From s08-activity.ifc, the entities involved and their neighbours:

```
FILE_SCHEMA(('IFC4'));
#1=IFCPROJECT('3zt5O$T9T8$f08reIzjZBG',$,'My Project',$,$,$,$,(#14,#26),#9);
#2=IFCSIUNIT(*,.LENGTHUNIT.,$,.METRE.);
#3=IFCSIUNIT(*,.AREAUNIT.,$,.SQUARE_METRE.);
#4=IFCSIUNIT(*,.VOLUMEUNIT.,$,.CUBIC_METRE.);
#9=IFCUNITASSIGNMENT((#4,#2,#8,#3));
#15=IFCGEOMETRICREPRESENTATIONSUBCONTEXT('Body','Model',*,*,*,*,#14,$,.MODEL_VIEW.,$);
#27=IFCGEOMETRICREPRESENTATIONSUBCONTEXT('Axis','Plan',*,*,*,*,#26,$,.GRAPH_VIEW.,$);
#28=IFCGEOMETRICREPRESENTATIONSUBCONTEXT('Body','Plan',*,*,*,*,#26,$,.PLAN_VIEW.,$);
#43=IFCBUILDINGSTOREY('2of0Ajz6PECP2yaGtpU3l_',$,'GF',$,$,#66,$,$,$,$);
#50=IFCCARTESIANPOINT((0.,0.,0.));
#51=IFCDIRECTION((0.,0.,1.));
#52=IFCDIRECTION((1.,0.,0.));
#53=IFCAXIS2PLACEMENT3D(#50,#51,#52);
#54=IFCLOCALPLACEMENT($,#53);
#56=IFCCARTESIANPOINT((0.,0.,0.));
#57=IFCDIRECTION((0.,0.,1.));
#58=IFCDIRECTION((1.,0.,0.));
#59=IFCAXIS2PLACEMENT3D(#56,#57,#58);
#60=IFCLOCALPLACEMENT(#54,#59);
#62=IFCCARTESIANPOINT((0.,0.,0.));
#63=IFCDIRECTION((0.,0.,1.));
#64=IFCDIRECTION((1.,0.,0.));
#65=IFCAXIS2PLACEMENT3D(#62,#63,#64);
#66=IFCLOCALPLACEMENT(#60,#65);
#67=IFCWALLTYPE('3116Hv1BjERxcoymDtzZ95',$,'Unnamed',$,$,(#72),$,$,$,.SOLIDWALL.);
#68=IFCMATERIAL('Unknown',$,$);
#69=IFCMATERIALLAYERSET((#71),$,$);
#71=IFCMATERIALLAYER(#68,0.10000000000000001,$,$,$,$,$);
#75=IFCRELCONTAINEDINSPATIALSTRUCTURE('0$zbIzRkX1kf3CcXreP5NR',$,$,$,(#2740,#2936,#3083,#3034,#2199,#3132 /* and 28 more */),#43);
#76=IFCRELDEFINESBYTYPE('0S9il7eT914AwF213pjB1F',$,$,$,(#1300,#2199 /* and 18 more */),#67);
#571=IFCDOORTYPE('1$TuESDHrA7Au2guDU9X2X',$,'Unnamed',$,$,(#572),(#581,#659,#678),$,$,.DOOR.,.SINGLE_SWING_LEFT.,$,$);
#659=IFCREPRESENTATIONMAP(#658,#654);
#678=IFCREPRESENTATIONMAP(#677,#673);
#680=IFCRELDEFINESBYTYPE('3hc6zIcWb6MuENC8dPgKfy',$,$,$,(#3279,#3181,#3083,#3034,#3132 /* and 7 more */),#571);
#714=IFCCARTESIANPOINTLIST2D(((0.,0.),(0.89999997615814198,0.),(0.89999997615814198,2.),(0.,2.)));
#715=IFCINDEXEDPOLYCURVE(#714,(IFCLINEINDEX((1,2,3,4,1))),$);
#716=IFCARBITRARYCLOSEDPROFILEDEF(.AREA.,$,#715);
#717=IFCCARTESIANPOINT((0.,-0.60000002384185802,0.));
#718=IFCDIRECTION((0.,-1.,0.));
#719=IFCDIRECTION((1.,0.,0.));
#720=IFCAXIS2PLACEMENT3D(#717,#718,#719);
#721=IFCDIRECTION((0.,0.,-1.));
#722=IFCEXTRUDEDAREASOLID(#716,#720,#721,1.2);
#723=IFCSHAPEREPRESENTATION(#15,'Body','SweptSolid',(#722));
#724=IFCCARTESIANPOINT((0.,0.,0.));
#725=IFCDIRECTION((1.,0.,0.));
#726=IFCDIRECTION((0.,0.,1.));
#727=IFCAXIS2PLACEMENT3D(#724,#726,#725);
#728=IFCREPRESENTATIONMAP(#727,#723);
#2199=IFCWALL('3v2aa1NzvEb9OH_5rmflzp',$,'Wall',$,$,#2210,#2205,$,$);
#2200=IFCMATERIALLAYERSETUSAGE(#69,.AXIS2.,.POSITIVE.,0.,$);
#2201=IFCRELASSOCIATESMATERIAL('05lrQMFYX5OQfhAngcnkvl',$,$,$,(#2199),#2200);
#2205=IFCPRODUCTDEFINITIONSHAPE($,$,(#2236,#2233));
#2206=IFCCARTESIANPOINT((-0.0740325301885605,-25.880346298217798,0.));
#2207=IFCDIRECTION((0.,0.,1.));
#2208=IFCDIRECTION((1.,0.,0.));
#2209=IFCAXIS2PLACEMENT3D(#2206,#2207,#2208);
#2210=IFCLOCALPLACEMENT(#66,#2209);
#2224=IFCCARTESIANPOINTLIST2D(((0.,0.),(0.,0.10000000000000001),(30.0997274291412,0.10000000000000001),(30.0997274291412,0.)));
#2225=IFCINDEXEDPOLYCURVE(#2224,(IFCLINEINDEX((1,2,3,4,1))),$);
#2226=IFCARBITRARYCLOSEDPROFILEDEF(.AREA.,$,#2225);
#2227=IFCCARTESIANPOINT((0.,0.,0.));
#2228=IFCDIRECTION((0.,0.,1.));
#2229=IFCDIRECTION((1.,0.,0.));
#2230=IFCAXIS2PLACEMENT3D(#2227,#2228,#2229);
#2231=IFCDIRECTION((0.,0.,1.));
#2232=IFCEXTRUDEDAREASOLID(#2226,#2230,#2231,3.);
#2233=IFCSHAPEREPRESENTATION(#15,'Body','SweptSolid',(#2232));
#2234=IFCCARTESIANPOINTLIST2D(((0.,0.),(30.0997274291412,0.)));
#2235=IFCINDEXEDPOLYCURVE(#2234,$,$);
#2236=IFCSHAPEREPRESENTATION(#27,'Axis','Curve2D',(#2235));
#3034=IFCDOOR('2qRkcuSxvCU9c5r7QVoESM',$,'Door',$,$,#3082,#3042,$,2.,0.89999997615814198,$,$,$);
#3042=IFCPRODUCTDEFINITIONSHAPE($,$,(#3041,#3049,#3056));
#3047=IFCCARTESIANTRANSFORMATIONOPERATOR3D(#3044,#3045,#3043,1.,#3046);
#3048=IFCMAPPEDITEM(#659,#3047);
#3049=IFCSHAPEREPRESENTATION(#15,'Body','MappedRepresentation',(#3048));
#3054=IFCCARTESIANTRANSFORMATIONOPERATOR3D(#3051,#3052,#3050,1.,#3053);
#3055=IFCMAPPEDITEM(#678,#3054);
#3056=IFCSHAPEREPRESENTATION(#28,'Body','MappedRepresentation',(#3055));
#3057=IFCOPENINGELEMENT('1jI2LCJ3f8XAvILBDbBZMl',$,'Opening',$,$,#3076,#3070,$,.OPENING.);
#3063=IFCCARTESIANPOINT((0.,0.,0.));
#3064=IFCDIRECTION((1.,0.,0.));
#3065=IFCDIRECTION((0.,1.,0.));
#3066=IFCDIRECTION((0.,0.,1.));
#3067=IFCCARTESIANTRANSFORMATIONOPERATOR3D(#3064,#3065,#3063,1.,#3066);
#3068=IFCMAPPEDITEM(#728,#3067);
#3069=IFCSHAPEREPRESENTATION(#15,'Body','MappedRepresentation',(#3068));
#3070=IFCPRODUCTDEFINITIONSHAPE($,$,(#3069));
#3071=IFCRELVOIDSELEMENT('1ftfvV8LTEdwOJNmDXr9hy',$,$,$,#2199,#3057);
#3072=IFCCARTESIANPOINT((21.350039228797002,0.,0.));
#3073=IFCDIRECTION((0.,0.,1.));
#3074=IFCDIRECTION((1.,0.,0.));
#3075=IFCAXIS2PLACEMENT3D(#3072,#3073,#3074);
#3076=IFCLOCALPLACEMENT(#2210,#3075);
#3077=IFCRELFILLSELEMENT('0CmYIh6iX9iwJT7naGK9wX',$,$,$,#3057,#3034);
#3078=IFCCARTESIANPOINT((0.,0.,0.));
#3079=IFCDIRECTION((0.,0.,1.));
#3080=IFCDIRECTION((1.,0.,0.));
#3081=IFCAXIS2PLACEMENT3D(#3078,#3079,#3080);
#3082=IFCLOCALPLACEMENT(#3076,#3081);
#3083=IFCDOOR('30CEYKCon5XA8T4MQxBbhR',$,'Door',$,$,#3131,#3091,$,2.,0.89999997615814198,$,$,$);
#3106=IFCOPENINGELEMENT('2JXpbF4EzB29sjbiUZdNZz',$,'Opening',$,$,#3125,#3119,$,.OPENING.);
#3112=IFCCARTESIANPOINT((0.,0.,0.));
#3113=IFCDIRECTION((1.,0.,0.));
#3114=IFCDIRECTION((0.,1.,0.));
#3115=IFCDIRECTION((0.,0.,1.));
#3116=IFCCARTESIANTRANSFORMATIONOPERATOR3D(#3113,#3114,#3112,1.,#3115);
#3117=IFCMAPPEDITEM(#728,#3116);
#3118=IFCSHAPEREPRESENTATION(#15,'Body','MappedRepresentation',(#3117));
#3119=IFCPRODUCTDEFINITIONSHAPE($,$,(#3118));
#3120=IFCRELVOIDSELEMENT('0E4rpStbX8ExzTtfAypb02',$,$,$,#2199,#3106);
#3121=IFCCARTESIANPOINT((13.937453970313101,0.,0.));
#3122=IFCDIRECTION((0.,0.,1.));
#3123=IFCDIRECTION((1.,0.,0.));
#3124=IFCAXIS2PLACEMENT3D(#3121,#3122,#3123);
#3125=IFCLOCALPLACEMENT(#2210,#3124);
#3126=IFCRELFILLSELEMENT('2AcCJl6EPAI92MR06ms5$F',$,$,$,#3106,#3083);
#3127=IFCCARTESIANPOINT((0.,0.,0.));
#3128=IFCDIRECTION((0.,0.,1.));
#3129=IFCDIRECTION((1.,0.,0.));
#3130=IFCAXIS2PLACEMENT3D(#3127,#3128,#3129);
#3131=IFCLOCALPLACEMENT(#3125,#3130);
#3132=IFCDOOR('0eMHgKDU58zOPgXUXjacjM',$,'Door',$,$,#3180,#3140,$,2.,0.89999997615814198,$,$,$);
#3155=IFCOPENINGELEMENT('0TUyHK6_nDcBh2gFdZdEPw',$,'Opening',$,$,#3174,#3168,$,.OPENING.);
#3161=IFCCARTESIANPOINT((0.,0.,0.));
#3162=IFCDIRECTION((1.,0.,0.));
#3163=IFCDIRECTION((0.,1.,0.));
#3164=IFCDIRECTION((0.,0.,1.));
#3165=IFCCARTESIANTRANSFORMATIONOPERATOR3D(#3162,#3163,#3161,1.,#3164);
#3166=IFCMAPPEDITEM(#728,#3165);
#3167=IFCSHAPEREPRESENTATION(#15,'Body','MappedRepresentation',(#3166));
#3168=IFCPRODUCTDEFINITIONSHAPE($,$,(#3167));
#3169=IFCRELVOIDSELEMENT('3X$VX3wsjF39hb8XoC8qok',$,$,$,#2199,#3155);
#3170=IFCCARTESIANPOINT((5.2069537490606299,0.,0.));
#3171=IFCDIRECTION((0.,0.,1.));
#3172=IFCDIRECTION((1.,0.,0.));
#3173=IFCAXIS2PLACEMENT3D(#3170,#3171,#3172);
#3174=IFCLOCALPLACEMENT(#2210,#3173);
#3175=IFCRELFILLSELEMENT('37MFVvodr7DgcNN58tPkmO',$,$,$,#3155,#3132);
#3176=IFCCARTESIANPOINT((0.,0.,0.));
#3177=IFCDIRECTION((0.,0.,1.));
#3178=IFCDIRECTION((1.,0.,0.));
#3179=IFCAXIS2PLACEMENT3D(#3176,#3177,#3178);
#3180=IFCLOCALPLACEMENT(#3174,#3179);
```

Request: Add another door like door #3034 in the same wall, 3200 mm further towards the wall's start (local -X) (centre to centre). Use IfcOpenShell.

```python
import ifcopenshell
import ifcopenshell.api.feature
import ifcopenshell.api.geometry
import ifcopenshell.api.root
import ifcopenshell.geom
import ifcopenshell.util.element
import ifcopenshell.util.placement
import ifcopenshell.util.shape
import ifcopenshell.util.unit

model = ifcopenshell.open("s08-activity.ifc")
unit_scale = ifcopenshell.util.unit.calculate_unit_scale(model)
settings = ifcopenshell.geom.settings()


def volume(element):
    """Net volume in cubic metres, openings subtracted."""
    shape = ifcopenshell.geom.create_shape(settings, element)
    return ifcopenshell.util.shape.get_volume(shape.geometry)


door = model.by_guid("2qRkcuSxvCU9c5r7QVoESM")
opening = door.FillsVoids[0].RelatingOpeningElement
wall = opening.VoidsElements[0].RelatingBuildingElement
before = volume(wall)
shift = ifcopenshell.util.placement.get_local_placement(wall.ObjectPlacement)[:3, 0] * -3.2 / unit_scale

# copy_class copies the void relationship, type, container and properties, but no geometry.
new_opening = ifcopenshell.api.root.copy_class(model, product=opening)
new_opening.Representation = ifcopenshell.util.element.copy_deep(
    model, opening.Representation, exclude=["IfcGeometricRepresentationContext", "IfcRepresentationMap"]
)
new_door = ifcopenshell.api.root.copy_class(model, product=door)
new_door.Representation = ifcopenshell.util.element.copy_deep(
    model, door.Representation, exclude=["IfcGeometricRepresentationContext", "IfcRepresentationMap"]
)
ifcopenshell.api.feature.add_filling(model, opening=new_opening, element=new_door)

for old, new in ((opening, new_opening), (door, new_door)):
    matrix = ifcopenshell.util.placement.get_local_placement(old.ObjectPlacement)
    matrix[:3, 3] += shift
    ifcopenshell.api.geometry.edit_object_placement(model, product=new, matrix=matrix, is_si=False)

after = volume(wall)

print(f"wall volume {before:.3f} -> {after:.3f} m3")

model.write("s08-activity-out.ifc")
```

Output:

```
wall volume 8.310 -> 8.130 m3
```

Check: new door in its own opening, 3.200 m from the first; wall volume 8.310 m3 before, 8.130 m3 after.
